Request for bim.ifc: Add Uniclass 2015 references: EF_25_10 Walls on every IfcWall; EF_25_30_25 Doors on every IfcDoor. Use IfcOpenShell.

First a look at what the model holds.

```python
import ifcopenshell

model = ifcopenshell.open("bim.ifc")
print(model.schema)
print("classifications:", [c.Name for c in model.by_type("IfcClassification")])
for ifc_class in ("IfcDoor", "IfcRoof", "IfcStair", "IfcWall", "IfcWindow"):
    print(ifc_class, len(model.by_type(ifc_class)))
```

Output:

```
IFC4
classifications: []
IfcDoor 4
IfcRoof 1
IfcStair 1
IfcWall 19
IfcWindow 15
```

```python
import ifcopenshell
import ifcopenshell.api.classification

model = ifcopenshell.open("bim.ifc")

system = ifcopenshell.api.classification.add_classification(model, classification="Uniclass 2015")

codes = {
    "IfcWall": ("EF_25_10", "Walls"),
    "IfcDoor": ("EF_25_30_25", "Doors"),
}
for ifc_class, (code, name) in codes.items():
    products = model.by_type(ifc_class)
    ifcopenshell.api.classification.add_reference(
        model, products=products, classification=system, identification=code, name=name
    )
    print(code, len(products))

model.write("bim-out.ifc")
```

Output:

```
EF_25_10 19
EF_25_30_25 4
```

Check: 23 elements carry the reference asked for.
